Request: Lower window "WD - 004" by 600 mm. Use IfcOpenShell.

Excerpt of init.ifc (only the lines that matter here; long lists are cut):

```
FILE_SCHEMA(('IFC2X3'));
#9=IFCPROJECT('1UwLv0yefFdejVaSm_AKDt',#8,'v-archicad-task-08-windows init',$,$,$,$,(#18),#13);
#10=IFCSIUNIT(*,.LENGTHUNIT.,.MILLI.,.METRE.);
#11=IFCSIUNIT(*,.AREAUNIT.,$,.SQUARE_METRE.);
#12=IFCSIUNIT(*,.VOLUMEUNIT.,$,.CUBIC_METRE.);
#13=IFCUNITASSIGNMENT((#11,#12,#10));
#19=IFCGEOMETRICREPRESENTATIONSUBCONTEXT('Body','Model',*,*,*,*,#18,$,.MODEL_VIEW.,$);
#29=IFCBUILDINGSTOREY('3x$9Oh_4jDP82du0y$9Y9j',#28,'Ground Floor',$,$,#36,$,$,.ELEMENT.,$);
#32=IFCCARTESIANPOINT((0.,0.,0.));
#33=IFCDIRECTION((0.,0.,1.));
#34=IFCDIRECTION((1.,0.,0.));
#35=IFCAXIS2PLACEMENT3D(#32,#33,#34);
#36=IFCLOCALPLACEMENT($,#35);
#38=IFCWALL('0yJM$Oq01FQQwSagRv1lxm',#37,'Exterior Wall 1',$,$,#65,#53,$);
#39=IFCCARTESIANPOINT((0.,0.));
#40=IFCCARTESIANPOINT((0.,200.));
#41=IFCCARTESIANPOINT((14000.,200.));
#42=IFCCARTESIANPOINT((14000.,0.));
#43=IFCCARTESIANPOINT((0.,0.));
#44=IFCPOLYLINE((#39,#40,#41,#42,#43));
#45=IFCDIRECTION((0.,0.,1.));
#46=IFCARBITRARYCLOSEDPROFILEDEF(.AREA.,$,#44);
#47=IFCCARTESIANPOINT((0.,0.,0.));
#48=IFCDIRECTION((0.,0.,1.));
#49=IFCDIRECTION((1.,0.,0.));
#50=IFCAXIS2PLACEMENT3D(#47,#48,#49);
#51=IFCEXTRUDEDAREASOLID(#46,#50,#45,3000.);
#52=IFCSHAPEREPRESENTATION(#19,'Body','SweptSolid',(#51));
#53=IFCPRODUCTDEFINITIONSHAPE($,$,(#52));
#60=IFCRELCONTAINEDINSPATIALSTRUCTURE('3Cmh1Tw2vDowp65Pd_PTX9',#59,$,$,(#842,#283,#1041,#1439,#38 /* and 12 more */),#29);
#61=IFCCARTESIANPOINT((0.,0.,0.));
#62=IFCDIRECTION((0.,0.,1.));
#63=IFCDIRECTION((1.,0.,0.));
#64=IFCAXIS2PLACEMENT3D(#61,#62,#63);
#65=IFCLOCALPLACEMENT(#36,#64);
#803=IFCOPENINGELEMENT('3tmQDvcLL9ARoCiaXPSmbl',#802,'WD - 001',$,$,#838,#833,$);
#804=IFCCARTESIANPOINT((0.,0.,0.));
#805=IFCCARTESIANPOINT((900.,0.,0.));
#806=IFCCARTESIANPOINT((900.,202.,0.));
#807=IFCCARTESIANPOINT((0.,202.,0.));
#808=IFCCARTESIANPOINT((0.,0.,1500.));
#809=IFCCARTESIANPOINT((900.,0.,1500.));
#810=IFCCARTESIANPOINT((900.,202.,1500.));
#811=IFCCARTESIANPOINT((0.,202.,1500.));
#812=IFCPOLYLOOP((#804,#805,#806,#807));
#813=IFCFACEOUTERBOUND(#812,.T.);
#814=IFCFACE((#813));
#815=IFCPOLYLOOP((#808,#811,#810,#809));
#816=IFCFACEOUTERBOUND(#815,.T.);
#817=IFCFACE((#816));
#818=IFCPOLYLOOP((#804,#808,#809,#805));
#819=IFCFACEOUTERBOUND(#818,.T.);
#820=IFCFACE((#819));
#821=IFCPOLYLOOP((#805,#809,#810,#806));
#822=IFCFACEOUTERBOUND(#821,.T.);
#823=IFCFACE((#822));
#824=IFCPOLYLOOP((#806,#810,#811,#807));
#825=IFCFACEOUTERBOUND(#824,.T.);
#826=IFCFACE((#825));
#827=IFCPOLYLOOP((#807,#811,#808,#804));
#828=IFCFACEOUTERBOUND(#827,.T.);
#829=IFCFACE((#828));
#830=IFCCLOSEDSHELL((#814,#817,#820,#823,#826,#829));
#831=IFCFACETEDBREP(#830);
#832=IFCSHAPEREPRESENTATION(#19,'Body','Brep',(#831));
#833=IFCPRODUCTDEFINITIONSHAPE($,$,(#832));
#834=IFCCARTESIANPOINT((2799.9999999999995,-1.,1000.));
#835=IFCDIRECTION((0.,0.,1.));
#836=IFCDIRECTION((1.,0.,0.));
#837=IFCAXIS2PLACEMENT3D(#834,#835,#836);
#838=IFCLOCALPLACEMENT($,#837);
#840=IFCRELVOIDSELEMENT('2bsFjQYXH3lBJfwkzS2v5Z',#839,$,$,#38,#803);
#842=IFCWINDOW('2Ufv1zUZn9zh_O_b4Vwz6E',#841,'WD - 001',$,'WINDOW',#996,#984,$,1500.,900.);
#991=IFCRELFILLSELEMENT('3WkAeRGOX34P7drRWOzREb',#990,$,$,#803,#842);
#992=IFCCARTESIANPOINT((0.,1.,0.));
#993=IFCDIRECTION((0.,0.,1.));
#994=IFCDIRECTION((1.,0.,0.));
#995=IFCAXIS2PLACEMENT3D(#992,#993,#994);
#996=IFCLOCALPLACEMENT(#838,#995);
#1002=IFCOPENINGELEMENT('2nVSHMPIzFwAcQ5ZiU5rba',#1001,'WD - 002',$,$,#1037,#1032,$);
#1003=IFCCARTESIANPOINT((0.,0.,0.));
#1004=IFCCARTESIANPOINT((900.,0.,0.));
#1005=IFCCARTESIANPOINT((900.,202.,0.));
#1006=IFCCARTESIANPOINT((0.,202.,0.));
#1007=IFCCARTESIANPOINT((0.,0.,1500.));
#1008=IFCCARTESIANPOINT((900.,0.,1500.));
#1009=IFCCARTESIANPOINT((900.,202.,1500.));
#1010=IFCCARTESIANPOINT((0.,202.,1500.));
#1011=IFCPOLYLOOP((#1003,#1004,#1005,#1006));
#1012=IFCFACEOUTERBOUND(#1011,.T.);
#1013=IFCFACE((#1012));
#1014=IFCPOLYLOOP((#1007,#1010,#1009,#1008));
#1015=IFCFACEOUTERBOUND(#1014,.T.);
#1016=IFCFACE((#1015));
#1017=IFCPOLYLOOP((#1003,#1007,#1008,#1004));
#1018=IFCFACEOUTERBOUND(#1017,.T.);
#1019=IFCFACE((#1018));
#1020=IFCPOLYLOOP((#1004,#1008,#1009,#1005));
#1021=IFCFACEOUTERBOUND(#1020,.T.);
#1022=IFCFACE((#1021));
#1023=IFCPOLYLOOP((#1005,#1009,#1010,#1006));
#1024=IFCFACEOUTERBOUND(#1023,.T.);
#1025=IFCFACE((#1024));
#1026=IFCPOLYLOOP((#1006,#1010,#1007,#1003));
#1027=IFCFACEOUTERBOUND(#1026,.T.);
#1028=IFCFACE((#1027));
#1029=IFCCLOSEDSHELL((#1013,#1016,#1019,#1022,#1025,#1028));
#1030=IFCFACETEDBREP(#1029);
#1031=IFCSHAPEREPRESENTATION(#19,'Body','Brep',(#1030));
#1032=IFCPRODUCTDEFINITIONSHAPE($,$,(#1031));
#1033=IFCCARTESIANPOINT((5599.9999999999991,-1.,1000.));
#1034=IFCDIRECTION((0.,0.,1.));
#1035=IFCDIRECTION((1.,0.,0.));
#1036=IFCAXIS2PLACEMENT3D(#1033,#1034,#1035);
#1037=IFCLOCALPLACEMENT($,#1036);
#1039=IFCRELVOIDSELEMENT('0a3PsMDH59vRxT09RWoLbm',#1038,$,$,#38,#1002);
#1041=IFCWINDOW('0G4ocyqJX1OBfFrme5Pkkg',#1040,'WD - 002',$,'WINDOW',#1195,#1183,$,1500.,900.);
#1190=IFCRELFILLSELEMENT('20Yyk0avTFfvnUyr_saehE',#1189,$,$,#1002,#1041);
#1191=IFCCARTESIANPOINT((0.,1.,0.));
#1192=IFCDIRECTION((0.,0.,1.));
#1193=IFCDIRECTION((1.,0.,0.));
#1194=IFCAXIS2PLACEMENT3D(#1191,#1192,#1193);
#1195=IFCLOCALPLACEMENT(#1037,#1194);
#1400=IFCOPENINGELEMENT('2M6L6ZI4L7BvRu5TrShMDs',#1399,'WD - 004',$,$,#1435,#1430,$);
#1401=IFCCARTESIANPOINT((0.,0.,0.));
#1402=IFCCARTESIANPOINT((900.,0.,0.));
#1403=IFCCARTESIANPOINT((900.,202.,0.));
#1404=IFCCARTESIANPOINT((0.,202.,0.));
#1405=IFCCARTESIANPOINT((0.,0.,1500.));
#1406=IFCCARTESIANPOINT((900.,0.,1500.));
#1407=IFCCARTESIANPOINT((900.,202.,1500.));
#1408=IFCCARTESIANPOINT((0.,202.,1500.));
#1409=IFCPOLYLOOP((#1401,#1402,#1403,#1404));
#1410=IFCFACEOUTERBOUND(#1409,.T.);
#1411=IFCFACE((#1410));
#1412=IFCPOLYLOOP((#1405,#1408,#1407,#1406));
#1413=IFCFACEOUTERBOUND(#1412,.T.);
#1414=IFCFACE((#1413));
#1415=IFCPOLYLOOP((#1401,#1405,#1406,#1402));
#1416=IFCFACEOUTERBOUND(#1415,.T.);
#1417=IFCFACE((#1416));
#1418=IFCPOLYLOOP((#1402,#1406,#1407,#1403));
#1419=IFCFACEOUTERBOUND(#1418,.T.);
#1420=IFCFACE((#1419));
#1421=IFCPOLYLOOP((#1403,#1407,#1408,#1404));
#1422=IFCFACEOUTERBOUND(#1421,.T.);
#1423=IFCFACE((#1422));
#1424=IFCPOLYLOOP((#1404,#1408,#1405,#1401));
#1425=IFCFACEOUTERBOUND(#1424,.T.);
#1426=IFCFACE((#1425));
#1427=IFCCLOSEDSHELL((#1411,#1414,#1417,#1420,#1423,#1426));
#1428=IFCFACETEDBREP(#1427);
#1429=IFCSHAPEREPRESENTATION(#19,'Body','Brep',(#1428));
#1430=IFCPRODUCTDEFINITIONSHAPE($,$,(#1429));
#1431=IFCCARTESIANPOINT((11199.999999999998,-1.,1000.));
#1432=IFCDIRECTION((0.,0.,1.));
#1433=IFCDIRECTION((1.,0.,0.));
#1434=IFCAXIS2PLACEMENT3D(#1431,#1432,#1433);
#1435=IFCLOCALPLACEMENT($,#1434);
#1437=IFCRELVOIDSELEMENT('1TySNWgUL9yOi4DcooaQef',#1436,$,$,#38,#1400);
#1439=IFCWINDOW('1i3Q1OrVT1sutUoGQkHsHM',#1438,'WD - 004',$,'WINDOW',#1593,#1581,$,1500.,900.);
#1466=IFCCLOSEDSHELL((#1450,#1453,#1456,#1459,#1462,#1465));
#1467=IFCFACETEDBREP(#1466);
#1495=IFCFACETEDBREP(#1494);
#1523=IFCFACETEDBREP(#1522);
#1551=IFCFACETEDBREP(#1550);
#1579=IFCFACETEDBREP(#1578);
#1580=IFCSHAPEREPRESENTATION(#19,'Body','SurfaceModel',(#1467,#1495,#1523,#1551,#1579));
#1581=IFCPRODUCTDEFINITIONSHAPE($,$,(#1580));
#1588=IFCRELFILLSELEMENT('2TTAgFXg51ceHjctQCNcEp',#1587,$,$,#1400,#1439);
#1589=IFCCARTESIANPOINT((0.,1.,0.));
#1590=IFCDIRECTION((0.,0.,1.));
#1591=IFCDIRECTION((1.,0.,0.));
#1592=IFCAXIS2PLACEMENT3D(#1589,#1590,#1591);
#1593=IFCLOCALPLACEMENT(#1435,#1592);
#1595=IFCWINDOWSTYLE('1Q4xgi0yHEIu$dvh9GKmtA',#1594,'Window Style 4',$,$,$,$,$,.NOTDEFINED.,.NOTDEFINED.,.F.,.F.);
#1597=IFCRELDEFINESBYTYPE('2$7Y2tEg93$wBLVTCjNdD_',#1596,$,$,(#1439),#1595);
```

```python
import numpy as np
import ifcopenshell
import ifcopenshell.api.geometry
import ifcopenshell.util.placement
import ifcopenshell.util.unit

model = ifcopenshell.open("init.ifc")
unit_scale = ifcopenshell.util.unit.calculate_unit_scale(model)

window = model.by_guid("1i3Q1OrVT1sutUoGQkHsHM")
opening = window.FillsVoids[0].RelatingOpeningElement
dz = -0.6 / unit_scale

shift = np.array([0.0, 0.0, dz])
# The window is placed relative to its opening, so it follows when the opening moves.
matrix = ifcopenshell.util.placement.get_local_placement(opening.ObjectPlacement)
matrix[:3, 3] += shift
ifcopenshell.api.geometry.edit_object_placement(
    model, product=opening, matrix=matrix, is_si=False, should_transform_children=True
)

print(f"moved by {dz * unit_scale:+.3f} m")

model.write("init_edited.ifc")
```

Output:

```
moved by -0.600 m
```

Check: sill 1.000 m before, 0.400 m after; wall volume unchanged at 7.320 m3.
